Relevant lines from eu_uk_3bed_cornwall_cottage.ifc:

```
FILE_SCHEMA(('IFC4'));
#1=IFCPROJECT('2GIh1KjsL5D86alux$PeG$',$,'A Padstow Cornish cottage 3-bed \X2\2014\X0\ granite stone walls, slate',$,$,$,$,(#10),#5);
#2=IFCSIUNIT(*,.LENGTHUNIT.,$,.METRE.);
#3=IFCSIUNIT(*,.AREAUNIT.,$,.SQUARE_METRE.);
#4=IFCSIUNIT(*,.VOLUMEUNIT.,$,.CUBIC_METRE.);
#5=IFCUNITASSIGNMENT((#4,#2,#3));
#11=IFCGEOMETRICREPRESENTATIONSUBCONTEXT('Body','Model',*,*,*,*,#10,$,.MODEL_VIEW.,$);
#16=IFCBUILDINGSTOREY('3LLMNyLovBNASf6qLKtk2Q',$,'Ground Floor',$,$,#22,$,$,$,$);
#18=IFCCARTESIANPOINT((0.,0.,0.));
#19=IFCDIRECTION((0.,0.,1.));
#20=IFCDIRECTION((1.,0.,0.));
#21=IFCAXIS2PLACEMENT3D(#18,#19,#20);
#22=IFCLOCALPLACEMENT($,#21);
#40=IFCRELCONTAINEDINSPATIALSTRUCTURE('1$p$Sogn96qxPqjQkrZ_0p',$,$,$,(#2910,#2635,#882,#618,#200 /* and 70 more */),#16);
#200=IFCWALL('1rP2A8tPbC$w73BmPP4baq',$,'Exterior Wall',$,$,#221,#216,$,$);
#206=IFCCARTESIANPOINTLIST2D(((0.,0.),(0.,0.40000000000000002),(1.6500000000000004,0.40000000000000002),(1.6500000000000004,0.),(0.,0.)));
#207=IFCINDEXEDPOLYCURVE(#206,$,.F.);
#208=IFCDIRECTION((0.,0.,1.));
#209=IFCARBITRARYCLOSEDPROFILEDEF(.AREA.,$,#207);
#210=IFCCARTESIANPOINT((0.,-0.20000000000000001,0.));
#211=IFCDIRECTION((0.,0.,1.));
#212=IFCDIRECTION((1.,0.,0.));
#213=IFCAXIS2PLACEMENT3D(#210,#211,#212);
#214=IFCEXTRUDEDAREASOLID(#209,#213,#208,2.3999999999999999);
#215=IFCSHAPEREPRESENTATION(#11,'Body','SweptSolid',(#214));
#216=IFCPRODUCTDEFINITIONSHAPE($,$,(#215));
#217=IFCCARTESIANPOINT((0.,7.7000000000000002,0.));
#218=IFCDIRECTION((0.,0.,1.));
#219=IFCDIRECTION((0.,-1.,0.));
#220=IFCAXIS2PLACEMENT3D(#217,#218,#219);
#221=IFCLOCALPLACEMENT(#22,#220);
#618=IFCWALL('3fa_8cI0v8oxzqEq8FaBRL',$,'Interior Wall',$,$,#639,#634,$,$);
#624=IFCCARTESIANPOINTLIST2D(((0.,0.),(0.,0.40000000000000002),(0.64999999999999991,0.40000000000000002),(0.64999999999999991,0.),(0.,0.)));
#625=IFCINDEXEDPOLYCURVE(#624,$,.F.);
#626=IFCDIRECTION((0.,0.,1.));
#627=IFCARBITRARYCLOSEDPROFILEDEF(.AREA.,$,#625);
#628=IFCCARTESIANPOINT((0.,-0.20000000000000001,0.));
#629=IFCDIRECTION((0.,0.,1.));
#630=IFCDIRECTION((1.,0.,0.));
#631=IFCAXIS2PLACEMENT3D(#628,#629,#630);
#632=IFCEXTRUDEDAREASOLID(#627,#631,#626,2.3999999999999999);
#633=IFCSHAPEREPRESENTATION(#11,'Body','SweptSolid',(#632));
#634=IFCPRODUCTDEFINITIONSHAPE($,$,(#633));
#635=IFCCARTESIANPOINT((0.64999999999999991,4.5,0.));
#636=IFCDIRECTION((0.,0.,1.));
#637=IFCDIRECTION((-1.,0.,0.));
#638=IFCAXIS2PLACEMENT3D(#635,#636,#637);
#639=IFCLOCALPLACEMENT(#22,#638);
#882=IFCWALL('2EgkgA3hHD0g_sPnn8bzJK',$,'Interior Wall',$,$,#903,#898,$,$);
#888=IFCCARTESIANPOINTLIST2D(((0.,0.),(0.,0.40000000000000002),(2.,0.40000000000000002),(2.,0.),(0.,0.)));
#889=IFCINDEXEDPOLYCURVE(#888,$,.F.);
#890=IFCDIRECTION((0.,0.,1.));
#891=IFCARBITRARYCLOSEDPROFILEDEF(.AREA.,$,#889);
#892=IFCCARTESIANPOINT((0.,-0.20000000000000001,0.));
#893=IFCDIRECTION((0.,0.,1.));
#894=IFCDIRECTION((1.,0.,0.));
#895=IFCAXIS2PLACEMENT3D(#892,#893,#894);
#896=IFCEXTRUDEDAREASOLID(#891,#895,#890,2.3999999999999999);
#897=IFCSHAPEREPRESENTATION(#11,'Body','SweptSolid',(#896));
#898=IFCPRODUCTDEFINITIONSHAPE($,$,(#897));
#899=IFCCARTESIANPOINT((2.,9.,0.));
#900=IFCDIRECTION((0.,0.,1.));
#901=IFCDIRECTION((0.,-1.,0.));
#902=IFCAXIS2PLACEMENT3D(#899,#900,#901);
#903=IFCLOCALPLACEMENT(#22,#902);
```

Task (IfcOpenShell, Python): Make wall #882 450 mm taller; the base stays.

```python
import ifcopenshell
import ifcopenshell.geom
import ifcopenshell.util.representation
import ifcopenshell.util.shape

model = ifcopenshell.open("eu_uk_3bed_cornwall_cottage.ifc")
settings = ifcopenshell.geom.settings()


def volume(element):
    """Net volume in cubic metres, openings subtracted."""
    shape = ifcopenshell.geom.create_shape(settings, element)
    return ifcopenshell.util.shape.get_volume(shape.geometry)


wall = model.by_id(882)
before = volume(wall)

body = ifcopenshell.util.representation.get_representation(wall, "Model", "Body")
solid = body.Items[0]
old_height = solid.Depth
solid.Depth += 0.45
after = volume(wall)

print(f"height {old_height:g} -> {solid.Depth:g}, volume {before:.3f} -> {after:.3f} m3")

model.write("eu_uk_3bed_cornwall_cottage_edited.ifc")
```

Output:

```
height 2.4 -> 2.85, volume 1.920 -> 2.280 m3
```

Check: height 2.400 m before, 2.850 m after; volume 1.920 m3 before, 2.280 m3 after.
